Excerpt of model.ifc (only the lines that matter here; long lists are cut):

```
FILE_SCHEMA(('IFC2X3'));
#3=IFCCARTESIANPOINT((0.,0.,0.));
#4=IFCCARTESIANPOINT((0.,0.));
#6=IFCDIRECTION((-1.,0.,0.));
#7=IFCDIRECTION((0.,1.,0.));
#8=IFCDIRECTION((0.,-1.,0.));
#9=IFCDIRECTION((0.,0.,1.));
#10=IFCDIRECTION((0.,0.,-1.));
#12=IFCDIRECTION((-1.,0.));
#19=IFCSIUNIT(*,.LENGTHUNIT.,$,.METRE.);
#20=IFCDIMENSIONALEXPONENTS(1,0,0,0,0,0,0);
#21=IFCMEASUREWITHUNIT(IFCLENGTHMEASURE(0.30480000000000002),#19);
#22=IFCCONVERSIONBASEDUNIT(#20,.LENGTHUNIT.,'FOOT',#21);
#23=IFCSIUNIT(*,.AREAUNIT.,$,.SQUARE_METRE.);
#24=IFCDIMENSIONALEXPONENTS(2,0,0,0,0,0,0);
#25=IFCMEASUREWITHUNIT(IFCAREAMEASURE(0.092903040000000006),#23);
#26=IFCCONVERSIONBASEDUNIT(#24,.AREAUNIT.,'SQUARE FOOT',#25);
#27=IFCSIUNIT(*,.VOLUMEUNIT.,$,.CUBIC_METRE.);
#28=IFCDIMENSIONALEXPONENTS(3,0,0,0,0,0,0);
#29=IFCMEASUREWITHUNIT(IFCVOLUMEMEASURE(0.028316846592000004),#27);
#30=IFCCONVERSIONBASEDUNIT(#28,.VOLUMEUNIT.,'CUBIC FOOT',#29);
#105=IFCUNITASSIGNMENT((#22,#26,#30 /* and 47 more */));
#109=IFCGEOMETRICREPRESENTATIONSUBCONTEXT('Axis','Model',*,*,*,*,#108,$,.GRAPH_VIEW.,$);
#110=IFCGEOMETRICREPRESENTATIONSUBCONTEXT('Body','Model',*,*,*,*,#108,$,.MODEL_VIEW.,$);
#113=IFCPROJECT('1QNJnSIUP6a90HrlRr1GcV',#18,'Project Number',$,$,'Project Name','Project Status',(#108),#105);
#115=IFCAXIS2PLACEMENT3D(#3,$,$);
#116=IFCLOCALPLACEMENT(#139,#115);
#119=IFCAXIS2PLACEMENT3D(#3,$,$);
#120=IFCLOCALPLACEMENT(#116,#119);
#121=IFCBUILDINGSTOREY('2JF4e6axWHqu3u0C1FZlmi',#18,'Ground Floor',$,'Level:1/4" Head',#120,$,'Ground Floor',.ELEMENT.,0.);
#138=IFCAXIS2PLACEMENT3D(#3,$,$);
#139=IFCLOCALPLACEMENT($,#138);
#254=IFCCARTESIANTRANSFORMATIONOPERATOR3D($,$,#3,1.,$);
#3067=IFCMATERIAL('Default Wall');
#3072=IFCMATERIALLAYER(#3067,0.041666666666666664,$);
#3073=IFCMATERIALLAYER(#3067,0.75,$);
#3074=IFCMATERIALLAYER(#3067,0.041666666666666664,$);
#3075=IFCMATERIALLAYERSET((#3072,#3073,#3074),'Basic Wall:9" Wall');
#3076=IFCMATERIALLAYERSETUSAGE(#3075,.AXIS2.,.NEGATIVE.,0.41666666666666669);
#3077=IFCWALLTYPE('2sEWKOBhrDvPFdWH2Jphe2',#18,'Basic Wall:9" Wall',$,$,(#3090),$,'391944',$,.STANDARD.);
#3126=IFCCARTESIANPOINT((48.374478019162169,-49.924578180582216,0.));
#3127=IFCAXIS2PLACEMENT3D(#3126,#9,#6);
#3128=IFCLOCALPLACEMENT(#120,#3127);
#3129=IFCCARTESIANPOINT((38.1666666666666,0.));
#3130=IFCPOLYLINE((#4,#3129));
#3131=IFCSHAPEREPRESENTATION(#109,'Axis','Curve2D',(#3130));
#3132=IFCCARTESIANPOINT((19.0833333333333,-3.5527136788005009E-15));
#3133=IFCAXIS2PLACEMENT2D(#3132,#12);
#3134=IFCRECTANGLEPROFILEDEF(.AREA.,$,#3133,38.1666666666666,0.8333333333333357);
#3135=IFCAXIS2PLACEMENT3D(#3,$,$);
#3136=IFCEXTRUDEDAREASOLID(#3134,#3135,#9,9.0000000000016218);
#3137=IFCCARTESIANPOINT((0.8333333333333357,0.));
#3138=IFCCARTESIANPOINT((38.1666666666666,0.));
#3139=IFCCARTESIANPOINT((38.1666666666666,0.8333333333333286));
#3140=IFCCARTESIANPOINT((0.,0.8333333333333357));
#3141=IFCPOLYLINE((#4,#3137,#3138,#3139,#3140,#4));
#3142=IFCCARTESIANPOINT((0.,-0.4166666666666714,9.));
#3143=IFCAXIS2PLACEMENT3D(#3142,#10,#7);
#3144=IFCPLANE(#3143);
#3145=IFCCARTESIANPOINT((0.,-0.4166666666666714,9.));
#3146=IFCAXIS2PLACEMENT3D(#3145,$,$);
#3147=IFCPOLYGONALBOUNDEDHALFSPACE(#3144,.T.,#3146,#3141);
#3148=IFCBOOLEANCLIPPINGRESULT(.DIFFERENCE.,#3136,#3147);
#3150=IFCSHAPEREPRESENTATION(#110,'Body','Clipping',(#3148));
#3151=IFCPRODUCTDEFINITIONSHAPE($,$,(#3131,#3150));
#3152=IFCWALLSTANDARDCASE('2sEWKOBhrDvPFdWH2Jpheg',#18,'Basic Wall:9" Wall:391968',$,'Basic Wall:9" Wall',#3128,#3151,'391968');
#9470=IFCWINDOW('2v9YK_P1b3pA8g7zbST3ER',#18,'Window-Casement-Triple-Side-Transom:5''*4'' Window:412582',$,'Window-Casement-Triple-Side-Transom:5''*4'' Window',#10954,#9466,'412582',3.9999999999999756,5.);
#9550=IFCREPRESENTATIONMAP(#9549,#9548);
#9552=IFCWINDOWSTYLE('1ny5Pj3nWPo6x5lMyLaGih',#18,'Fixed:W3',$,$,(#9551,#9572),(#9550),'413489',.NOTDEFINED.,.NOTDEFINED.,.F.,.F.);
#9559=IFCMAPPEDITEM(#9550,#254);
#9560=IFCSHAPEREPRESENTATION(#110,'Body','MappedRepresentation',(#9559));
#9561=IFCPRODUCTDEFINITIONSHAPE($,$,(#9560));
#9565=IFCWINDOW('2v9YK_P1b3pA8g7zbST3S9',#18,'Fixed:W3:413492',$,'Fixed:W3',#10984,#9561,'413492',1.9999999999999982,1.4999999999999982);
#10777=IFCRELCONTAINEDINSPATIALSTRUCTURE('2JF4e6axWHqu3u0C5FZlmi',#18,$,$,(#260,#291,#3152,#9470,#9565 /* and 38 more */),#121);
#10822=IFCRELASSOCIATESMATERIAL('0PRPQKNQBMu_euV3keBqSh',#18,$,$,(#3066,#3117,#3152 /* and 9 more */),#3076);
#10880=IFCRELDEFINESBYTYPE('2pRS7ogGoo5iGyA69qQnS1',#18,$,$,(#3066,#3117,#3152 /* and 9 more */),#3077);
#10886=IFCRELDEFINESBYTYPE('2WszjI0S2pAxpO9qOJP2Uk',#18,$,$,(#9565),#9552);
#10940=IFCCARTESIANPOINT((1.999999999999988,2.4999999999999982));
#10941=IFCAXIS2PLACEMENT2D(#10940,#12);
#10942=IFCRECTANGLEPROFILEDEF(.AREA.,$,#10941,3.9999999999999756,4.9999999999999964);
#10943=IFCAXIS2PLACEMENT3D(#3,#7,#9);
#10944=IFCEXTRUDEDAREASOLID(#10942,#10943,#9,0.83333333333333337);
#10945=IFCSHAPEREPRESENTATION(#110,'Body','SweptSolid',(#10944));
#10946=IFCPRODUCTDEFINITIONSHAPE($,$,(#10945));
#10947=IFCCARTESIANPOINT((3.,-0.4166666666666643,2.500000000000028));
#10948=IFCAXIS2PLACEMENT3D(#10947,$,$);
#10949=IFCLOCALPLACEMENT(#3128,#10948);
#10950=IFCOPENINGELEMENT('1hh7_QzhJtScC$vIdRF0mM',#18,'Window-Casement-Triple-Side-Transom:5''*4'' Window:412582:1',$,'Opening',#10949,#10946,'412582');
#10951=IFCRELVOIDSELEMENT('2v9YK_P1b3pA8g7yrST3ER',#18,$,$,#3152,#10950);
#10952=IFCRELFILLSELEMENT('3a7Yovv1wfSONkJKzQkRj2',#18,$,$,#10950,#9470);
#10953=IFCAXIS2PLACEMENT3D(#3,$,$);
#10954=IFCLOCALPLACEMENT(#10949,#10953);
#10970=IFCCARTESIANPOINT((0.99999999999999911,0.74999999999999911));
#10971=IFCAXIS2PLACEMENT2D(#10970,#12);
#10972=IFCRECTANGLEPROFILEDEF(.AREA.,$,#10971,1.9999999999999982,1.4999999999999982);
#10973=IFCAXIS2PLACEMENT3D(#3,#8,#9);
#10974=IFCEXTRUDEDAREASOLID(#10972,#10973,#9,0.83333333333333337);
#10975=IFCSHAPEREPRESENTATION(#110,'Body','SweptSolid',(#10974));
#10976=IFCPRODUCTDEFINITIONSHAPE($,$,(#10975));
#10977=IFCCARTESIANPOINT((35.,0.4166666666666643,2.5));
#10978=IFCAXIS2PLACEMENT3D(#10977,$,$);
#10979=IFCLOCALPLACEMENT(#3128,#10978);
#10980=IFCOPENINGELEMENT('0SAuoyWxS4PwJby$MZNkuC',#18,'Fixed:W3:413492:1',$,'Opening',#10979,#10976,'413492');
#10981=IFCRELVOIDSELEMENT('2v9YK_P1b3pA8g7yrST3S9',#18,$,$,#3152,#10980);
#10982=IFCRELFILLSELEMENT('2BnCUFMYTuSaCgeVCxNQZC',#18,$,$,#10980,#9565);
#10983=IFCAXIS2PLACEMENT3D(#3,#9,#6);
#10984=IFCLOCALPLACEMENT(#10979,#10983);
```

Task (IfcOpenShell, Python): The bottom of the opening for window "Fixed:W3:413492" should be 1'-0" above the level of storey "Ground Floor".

```python
import numpy as np
import ifcopenshell
import ifcopenshell.api.geometry
import ifcopenshell.geom
import ifcopenshell.util.element
import ifcopenshell.util.placement
import ifcopenshell.util.shape
import ifcopenshell.util.unit

model = ifcopenshell.open("model.ifc")
unit_scale = ifcopenshell.util.unit.calculate_unit_scale(model)

window = model.by_guid("2v9YK_P1b3pA8g7zbST3S9")
opening = window.FillsVoids[0].RelatingOpeningElement
storey = ifcopenshell.util.element.get_container(window, ifc_class="IfcBuildingStorey")
level = ifcopenshell.util.placement.get_local_placement(storey.ObjectPlacement)[2, 3]

# The opening's origin need not be at the sill, so measure its lowest point.
shape = ifcopenshell.geom.create_shape(ifcopenshell.geom.settings(), opening)
bottom = ifcopenshell.util.shape.get_shape_bottom_elevation(shape, shape.geometry) / unit_scale
dz = level + 12 * 0.0254 / unit_scale - bottom

shift = np.array([0.0, 0.0, dz])
# The window is placed relative to its opening, so it follows when the opening moves.
matrix = ifcopenshell.util.placement.get_local_placement(opening.ObjectPlacement)
matrix[:3, 3] += shift
ifcopenshell.api.geometry.edit_object_placement(
    model, product=opening, matrix=matrix, is_si=False, should_transform_children=True
)

print(f"moved by {dz * unit_scale:+.3f} m")

model.write("model_updated.ifc")
```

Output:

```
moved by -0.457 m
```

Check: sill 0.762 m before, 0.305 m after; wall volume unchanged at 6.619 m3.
